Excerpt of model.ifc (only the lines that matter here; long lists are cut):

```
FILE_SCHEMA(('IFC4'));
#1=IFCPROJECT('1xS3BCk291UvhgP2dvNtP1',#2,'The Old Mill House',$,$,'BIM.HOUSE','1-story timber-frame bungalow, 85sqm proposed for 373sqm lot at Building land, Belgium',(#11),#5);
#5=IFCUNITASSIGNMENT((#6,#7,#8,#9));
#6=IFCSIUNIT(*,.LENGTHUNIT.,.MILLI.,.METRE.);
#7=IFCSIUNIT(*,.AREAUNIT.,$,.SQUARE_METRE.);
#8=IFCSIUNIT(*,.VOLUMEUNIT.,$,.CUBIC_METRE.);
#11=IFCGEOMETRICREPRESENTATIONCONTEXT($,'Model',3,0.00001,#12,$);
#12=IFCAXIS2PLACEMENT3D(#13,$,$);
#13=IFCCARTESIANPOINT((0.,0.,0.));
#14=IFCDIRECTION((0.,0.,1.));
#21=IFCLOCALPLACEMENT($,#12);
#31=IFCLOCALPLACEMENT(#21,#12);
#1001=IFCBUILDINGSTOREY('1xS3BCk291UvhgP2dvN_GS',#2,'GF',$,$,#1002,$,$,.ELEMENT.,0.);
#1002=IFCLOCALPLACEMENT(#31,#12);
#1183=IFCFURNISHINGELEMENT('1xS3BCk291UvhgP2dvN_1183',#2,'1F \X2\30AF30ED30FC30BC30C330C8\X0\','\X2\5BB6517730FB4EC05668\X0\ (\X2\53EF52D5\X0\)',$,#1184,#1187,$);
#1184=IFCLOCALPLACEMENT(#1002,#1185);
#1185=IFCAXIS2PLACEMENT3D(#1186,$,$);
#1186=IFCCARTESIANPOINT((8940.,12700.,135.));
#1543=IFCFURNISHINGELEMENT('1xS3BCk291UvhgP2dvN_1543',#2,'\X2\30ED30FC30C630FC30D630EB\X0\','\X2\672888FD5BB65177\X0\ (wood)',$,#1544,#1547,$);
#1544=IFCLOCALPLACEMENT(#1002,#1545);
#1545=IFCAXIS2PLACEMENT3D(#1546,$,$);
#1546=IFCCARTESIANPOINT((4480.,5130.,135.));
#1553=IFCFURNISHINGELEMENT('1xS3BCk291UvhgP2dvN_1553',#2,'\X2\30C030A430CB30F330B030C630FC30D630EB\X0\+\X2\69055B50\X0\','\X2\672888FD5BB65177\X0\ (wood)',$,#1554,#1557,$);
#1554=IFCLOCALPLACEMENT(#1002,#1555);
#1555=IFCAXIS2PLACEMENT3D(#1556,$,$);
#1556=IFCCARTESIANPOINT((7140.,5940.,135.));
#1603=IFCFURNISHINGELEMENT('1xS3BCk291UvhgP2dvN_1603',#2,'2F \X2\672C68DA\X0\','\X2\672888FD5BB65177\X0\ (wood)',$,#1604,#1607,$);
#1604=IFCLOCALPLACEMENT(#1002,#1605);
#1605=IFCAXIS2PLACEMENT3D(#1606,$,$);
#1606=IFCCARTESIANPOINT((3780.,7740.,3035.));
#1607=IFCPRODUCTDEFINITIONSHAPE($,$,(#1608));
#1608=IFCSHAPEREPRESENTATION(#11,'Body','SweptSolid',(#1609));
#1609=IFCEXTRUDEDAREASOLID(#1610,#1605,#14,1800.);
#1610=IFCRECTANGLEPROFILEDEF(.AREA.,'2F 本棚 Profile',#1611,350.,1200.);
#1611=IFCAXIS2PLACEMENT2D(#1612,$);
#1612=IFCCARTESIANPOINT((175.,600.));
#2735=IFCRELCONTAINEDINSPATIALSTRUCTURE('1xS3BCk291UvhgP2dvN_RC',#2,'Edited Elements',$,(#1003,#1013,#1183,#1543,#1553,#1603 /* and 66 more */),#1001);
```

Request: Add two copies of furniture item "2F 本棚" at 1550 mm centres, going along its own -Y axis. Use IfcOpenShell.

```python
import ifcopenshell
import ifcopenshell.api.geometry
import ifcopenshell.api.root
import ifcopenshell.util.element
import ifcopenshell.util.placement

model = ifcopenshell.open("model.ifc")


def reuse_history(source, copy):
    """copy_class also copies each property set's owner history, people and application; keep the originals."""
    for rel in copy.IsDefinedBy:
        if rel.is_a("IfcRelDefinesByProperties") and (history := rel.RelatingPropertyDefinition.OwnerHistory):
            rel.RelatingPropertyDefinition.OwnerHistory = source.OwnerHistory
            ifcopenshell.util.element.remove_deep2(model, history)


source = model.by_guid("1xS3BCk291UvhgP2dvN_1603")
base = ifcopenshell.util.placement.get_local_placement(source.ObjectPlacement)
step = -base[:3, 1] * 1550.0

for i in range(1, 3):
    copy = ifcopenshell.api.root.copy_class(model, product=source)
    copy.Representation = ifcopenshell.util.element.copy_deep(
        model, source.Representation, exclude=["IfcGeometricRepresentationContext", "IfcRepresentationMap"]
    )
    reuse_history(source, copy)
    matrix = base.copy()
    matrix[:3, 3] += i * step
    print("added at", matrix[:3, 3].round(3) + 0.0)
    ifcopenshell.api.geometry.edit_object_placement(model, product=copy, matrix=matrix, is_si=False)

model.write("model_v2.ifc")
```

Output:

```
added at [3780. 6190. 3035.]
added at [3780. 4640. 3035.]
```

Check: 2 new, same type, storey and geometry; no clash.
